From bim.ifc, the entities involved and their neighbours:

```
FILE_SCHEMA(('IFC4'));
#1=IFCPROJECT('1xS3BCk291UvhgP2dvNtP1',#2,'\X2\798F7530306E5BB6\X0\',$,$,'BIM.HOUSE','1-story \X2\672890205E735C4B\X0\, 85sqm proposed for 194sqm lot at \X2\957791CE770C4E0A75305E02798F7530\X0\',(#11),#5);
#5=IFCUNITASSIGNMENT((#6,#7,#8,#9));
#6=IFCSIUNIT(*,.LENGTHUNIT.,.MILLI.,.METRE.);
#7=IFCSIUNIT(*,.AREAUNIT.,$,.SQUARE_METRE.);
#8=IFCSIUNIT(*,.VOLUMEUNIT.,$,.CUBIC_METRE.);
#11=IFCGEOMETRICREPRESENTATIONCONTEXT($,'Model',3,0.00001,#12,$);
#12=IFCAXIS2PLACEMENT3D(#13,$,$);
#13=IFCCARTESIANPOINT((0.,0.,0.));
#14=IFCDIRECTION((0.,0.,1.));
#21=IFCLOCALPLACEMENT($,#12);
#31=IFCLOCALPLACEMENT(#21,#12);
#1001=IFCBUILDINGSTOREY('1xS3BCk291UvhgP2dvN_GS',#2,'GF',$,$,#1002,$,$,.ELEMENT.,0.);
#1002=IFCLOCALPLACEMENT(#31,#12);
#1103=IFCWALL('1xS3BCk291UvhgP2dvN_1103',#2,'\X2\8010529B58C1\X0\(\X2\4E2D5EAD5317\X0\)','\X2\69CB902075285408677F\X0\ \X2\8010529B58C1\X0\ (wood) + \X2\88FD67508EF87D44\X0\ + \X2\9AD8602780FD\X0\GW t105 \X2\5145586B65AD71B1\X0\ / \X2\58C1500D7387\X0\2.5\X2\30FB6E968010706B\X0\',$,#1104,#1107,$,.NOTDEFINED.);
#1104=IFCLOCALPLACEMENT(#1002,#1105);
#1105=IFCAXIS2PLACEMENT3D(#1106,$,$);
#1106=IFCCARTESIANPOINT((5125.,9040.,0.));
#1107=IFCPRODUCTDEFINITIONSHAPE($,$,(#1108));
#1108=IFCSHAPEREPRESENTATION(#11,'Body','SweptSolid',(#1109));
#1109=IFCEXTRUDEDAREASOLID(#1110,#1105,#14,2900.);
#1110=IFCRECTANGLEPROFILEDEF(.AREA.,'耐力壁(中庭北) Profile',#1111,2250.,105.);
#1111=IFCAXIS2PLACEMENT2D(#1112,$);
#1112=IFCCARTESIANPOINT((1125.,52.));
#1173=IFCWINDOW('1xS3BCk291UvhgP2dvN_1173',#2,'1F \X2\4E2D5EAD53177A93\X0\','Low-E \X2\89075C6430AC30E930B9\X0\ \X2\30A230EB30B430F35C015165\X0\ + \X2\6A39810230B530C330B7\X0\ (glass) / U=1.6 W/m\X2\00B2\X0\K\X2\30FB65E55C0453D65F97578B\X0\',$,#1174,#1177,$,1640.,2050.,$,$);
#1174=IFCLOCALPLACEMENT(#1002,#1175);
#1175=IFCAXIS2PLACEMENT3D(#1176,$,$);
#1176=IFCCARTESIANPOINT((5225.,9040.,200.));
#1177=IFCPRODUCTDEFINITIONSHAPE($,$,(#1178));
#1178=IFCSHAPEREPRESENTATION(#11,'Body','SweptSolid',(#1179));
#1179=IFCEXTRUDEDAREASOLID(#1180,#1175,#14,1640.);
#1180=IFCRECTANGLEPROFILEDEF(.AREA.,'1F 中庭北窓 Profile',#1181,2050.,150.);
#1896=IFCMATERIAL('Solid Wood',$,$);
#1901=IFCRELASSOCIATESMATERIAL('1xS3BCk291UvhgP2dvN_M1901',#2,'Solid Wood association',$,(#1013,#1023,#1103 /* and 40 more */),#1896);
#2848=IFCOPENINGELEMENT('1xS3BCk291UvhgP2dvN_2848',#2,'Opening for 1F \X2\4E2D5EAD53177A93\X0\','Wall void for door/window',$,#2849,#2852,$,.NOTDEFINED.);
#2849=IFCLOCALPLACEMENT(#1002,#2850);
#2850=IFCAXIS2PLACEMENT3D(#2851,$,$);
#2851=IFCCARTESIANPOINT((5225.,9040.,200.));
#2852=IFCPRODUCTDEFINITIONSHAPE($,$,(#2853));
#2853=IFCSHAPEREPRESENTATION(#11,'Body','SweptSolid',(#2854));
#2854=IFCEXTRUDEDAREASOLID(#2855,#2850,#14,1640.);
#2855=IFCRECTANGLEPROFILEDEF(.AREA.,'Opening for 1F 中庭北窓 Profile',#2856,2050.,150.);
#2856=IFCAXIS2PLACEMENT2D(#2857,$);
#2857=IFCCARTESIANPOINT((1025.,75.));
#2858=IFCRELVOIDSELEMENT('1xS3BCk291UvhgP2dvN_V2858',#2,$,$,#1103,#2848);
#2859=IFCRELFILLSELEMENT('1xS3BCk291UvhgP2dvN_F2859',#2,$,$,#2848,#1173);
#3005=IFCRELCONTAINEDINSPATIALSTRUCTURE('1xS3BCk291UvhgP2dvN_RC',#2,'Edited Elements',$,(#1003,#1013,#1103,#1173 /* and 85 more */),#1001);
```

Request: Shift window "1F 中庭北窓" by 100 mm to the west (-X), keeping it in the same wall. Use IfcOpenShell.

```python
import ifcopenshell
import ifcopenshell.api.geometry
import ifcopenshell.util.placement

model = ifcopenshell.open("bim.ifc")

window = model.by_guid("1xS3BCk291UvhgP2dvN_1173")
opening = window.FillsVoids[0].RelatingOpeningElement
wall = opening.VoidsElements[0].RelatingBuildingElement

wall_matrix = ifcopenshell.util.placement.get_local_placement(wall.ObjectPlacement)
shift = wall_matrix[:3, 0] * -100.0
before = ifcopenshell.util.placement.get_local_placement(window.ObjectPlacement)[:3, 3].copy()

# The window is not placed relative to its opening, so move both.
for product in (opening, window):
    matrix = ifcopenshell.util.placement.get_local_placement(product.ObjectPlacement)
    matrix[:3, 3] += shift
    ifcopenshell.api.geometry.edit_object_placement(model, product=product, matrix=matrix, is_si=False)

after = ifcopenshell.util.placement.get_local_placement(window.ObjectPlacement)[:3, 3]
print("window moved by", (after - before).round(3) + 0.0)

model.write("bim_updated.ifc")
```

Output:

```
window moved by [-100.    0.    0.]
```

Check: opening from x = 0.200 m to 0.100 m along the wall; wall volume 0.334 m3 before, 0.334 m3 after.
